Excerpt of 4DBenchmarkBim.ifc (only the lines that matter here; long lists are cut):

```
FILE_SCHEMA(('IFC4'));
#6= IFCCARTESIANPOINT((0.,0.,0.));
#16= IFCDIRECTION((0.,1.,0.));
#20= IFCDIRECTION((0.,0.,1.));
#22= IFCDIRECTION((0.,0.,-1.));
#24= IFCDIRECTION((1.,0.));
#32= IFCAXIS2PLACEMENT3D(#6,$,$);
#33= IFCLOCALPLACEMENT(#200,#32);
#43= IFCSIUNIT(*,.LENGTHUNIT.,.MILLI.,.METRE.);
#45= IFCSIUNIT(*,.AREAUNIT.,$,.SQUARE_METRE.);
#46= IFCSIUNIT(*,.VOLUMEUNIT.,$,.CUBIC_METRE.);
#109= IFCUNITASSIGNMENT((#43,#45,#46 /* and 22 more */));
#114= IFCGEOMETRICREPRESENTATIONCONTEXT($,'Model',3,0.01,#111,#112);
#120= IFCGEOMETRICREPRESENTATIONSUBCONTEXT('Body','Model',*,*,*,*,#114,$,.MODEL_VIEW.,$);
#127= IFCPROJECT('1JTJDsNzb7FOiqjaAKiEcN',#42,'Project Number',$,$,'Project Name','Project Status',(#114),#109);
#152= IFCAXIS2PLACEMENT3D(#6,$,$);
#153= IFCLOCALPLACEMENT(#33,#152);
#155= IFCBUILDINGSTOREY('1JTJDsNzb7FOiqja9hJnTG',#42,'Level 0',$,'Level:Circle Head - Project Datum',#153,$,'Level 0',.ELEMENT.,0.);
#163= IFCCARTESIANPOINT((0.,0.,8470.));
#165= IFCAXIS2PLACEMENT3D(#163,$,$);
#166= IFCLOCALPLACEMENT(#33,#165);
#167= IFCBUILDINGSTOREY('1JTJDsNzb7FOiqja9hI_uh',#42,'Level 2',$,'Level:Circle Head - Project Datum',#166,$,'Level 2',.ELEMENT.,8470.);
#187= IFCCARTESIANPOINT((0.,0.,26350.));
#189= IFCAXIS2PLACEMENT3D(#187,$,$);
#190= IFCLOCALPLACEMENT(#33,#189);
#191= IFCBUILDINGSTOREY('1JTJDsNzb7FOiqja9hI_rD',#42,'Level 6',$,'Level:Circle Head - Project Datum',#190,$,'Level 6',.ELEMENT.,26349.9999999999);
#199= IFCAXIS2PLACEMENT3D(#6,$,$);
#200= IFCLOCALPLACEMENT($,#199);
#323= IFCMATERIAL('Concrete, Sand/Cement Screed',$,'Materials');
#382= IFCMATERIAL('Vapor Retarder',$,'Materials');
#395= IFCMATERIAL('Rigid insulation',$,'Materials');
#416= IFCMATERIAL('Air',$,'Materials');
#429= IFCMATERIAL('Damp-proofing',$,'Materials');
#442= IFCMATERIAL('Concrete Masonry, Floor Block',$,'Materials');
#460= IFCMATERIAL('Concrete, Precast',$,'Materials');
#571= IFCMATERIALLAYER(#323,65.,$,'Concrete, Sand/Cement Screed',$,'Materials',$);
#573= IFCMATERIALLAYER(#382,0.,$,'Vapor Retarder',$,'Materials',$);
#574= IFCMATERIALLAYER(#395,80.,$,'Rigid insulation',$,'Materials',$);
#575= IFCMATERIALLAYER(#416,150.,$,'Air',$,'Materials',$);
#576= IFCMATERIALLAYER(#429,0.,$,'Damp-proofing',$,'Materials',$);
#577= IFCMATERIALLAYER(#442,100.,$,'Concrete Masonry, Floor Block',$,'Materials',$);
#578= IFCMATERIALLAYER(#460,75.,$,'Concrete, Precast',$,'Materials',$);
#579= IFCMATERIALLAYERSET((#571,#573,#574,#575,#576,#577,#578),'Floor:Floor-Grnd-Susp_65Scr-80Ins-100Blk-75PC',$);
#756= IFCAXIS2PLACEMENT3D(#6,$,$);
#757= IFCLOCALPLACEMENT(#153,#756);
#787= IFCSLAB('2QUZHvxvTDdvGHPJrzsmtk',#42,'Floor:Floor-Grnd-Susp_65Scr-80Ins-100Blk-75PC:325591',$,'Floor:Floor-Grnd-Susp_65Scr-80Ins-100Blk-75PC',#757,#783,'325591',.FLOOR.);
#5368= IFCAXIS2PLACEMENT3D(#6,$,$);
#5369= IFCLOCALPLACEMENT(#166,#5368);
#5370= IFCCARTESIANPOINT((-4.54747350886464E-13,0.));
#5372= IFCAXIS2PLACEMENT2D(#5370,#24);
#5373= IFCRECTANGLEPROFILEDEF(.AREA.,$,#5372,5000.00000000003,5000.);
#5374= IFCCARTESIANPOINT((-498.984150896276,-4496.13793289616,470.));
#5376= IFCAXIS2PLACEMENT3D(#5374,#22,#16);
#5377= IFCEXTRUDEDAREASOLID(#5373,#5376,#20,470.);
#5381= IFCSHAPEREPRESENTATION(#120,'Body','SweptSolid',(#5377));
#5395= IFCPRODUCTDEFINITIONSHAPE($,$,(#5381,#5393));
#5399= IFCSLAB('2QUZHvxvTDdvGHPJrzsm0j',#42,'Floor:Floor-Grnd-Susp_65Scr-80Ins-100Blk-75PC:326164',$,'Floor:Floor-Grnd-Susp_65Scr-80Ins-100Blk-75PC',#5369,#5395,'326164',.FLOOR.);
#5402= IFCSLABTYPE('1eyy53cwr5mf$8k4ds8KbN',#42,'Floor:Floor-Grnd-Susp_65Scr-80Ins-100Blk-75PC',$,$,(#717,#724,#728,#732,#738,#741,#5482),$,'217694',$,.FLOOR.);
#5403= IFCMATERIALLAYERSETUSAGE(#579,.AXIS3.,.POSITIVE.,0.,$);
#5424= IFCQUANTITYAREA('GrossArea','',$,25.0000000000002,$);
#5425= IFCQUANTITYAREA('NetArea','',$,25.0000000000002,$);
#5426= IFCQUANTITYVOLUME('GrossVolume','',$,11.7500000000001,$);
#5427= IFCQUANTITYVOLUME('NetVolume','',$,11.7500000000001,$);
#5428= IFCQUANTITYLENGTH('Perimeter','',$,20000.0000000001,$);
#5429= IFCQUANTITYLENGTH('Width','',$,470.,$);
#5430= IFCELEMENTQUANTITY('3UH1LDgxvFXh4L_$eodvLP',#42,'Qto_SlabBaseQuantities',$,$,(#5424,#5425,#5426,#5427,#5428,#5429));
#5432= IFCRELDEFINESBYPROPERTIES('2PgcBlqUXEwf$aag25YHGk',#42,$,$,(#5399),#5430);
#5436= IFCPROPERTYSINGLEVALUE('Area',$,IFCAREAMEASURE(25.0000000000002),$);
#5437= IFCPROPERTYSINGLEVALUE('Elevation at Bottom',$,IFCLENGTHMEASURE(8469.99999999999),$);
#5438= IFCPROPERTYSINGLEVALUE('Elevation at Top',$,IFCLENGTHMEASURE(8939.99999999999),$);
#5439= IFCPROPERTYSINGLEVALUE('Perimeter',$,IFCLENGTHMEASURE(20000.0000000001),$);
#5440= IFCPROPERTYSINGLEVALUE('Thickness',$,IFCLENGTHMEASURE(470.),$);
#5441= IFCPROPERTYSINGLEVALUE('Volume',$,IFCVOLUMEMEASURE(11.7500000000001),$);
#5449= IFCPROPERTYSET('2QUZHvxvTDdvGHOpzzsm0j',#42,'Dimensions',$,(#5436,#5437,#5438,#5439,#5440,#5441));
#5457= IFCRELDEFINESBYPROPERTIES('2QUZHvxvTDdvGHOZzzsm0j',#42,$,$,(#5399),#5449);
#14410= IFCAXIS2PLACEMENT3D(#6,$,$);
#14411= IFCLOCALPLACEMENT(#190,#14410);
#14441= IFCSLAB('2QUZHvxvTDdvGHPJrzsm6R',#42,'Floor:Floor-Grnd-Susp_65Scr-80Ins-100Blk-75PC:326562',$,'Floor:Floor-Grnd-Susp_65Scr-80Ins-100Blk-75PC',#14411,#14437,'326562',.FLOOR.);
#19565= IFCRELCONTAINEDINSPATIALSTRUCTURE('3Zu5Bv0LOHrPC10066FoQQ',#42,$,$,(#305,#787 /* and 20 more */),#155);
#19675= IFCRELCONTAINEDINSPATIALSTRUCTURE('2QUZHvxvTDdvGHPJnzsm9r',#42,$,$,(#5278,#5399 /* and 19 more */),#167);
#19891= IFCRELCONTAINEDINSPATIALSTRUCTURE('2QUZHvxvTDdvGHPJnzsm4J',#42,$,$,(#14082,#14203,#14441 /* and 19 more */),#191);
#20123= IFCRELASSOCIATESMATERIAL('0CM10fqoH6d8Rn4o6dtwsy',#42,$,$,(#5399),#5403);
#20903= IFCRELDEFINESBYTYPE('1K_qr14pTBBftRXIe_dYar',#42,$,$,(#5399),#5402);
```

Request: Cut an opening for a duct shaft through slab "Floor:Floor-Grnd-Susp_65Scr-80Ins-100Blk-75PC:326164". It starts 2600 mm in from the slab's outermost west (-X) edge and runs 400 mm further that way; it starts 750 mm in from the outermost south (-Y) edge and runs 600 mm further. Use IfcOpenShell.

```python
import numpy as np
import ifcopenshell
import ifcopenshell.api.feature
import ifcopenshell.api.geometry
import ifcopenshell.api.pset
import ifcopenshell.api.root
import ifcopenshell.geom
import ifcopenshell.util.element
import ifcopenshell.util.placement
import ifcopenshell.util.representation
import ifcopenshell.util.shape
import ifcopenshell.util.unit

model = ifcopenshell.open("4DBenchmarkBim.ifc")
unit_scale = ifcopenshell.util.unit.calculate_unit_scale(model)
area_scale = ifcopenshell.util.unit.calculate_unit_scale(model, "AREAUNIT")
volume_scale = ifcopenshell.util.unit.calculate_unit_scale(model, "VOLUMEUNIT")
settings = ifcopenshell.geom.settings()


def volume(element):
    """Net volume in cubic metres, openings subtracted."""
    shape = ifcopenshell.geom.create_shape(settings, element)
    return ifcopenshell.util.shape.get_volume(shape.geometry)


slab = model.by_guid("2QUZHvxvTDdvGHPJrzsm0j")
before = volume(slab)

# Extent in the slab's own axes, in metres. The edges named are its -X and -Y sides.
slab_shape = ifcopenshell.geom.create_shape(settings, slab)
vertices = ifcopenshell.util.shape.get_vertices(slab_shape.geometry)
x_min, y_min, bottom = vertices.min(axis=0)
top = vertices[:, 2].max()

opening = ifcopenshell.api.root.create_entity(model, ifc_class="IfcOpeningElement", name="Duct shaft opening", predefined_type="OPENING")
context = ifcopenshell.util.representation.get_context(model, "Model", "Body", "MODEL_VIEW")
width, depth = 0.4, 0.6
outline = [(0.0, 0.0), (width, 0.0), (width, depth), (0.0, depth), (0.0, 0.0)]
# Overshoot both faces by 50 mm so the cut is clean.
shape = ifcopenshell.api.geometry.add_slab_representation(
    model, context=context, depth=top - bottom + 0.1, polyline=outline
)
ifcopenshell.api.geometry.assign_representation(model, product=opening, representation=shape)

matrix = ifcopenshell.util.placement.get_local_placement(slab.ObjectPlacement)
matrix[:, 3] = matrix @ np.append(np.array([x_min + 2.6, y_min + 0.75, bottom - 0.05]) / unit_scale, 1.0)
ifcopenshell.api.geometry.edit_object_placement(model, product=opening, matrix=matrix, is_si=False)
ifcopenshell.api.feature.add_feature(model, feature=opening, element=slab)

after = volume(slab)

# Update the slab's stored quantities.
qto = model.by_id(ifcopenshell.util.element.get_pset(slab, "Qto_SlabBaseQuantities", should_inherit=False)["id"])
ifcopenshell.api.pset.edit_qto(model, qto=qto, properties={
    "NetArea": after / (top - bottom) / area_scale,
    "NetVolume": after / volume_scale,
})
pset = model.by_id(ifcopenshell.util.element.get_pset(slab, "Dimensions", should_inherit=False)["id"])
ifcopenshell.api.pset.edit_pset(model, pset=pset, properties={
    "Area": model.create_entity("IfcAreaMeasure", after / (top - bottom) / area_scale),
    "Volume": model.create_entity("IfcVolumeMeasure", after / volume_scale),
})

print(f"slab volume {before:.3f} -> {after:.3f} m3")

model.write("4DBenchmarkBim-out.ifc")
```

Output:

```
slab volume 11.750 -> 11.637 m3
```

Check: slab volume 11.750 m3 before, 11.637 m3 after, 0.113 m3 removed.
